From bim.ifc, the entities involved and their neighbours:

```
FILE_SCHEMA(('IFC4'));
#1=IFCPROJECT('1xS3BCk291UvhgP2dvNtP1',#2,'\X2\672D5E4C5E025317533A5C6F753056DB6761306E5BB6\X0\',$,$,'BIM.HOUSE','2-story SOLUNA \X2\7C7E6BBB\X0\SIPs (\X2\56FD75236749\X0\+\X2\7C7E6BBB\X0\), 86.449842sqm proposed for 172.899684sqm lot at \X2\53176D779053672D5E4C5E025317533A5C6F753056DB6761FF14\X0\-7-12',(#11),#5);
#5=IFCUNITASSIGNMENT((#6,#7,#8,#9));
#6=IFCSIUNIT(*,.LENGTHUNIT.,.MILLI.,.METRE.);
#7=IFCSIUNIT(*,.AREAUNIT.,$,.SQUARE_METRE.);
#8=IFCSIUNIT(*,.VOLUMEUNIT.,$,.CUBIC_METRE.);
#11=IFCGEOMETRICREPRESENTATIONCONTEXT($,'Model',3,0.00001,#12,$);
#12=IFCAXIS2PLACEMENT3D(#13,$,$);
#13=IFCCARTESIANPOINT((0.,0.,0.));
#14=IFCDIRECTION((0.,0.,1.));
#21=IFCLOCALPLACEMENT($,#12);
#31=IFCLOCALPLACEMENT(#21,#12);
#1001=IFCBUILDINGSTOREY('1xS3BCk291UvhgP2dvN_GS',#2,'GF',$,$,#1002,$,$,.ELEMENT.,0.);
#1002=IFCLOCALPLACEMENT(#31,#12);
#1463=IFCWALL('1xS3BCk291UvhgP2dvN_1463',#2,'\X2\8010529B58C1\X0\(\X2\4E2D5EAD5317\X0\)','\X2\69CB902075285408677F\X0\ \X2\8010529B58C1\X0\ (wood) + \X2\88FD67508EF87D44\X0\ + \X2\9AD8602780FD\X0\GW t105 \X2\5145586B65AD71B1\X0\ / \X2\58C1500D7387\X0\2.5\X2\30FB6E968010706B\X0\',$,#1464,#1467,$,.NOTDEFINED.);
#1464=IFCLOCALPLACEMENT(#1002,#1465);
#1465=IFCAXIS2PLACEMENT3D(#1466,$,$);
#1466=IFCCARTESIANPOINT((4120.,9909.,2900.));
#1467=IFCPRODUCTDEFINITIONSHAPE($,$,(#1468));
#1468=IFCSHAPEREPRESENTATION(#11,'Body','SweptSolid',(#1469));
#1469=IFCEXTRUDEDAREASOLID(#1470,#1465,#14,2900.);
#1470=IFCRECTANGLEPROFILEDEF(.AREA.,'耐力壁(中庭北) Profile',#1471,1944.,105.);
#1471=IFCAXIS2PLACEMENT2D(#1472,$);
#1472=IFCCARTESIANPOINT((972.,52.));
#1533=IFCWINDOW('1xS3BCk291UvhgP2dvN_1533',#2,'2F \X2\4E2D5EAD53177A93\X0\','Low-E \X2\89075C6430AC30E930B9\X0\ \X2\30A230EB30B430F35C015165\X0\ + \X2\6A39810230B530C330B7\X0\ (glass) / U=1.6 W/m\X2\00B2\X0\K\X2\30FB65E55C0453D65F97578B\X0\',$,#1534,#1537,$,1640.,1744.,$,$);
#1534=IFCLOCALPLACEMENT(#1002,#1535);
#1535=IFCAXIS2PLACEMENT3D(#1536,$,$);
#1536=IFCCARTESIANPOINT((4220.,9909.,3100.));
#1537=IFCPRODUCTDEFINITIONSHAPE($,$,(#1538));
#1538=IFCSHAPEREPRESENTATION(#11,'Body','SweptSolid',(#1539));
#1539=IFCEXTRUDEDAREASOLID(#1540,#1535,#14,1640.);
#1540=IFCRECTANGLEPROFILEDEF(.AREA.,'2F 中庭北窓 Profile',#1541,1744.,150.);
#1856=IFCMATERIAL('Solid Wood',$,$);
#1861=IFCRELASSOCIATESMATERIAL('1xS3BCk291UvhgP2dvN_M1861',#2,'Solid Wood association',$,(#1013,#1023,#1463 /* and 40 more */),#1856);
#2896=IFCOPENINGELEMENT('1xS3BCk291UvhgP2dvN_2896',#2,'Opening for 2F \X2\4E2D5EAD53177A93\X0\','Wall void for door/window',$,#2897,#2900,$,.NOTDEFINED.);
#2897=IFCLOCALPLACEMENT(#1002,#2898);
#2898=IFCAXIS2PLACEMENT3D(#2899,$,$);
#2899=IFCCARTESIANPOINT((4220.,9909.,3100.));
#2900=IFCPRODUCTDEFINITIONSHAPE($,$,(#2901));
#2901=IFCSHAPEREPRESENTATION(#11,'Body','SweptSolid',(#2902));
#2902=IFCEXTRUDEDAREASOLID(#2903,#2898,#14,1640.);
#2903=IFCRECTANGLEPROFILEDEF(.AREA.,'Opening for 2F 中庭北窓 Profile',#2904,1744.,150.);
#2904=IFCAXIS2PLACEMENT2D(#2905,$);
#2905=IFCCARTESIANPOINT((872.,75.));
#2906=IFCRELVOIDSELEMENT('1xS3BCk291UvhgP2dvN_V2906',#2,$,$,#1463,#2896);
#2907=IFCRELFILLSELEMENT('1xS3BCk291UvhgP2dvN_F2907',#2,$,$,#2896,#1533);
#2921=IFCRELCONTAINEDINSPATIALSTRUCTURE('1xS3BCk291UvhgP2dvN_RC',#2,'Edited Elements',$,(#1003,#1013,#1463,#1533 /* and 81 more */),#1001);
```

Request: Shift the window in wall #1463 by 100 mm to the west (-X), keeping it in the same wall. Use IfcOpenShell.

```python
import ifcopenshell
import ifcopenshell.api.geometry
import ifcopenshell.util.placement

model = ifcopenshell.open("bim.ifc")

window = model.by_guid("1xS3BCk291UvhgP2dvN_1533")
opening = window.FillsVoids[0].RelatingOpeningElement
wall = opening.VoidsElements[0].RelatingBuildingElement

wall_matrix = ifcopenshell.util.placement.get_local_placement(wall.ObjectPlacement)
shift = wall_matrix[:3, 0] * -100.0
before = ifcopenshell.util.placement.get_local_placement(window.ObjectPlacement)[:3, 3].copy()

# The window is not placed relative to its opening, so move both.
for product in (opening, window):
    matrix = ifcopenshell.util.placement.get_local_placement(product.ObjectPlacement)
    matrix[:3, 3] += shift
    ifcopenshell.api.geometry.edit_object_placement(model, product=product, matrix=matrix, is_si=False)

after = ifcopenshell.util.placement.get_local_placement(window.ObjectPlacement)[:3, 3]
print("window moved by", (after - before).round(3) + 0.0)

model.write("bim_edited.ifc")
```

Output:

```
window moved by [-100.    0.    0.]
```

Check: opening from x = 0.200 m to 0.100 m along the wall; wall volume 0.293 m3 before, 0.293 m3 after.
